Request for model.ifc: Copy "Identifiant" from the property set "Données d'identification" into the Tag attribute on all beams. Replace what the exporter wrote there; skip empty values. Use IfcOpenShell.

First a look at what the model holds.

```python
import ifcopenshell
import ifcopenshell.util.element

model = ifcopenshell.open("model.ifc")
print(model.schema)
beams = model.by_type("IfcBeam")
print(len(beams), "beams")
for e in beams[:8]:
    source = ifcopenshell.util.element.get_pset(e, "Données d'identification", "Identifiant")
    target = e.Tag
    print(e.id(), repr(source), repr(target), sep=" | ")
```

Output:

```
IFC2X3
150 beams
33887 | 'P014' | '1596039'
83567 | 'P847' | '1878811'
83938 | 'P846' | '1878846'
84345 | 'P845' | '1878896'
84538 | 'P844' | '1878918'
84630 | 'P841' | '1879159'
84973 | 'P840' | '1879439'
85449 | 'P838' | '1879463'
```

```python
import ifcopenshell
import ifcopenshell.util.element

model = ifcopenshell.open("model.ifc")

count = 0
for e in model.by_type("IfcBeam"):
    value = ifcopenshell.util.element.get_pset(e, "Données d'identification", "Identifiant")
    current = e.Tag
    if not value or not value.strip() or current == value:
        continue
    e.Tag = value
    count += 1

print(count, "beams updated")

model.write("model_v2.ifc")
```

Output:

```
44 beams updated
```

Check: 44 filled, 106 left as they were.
